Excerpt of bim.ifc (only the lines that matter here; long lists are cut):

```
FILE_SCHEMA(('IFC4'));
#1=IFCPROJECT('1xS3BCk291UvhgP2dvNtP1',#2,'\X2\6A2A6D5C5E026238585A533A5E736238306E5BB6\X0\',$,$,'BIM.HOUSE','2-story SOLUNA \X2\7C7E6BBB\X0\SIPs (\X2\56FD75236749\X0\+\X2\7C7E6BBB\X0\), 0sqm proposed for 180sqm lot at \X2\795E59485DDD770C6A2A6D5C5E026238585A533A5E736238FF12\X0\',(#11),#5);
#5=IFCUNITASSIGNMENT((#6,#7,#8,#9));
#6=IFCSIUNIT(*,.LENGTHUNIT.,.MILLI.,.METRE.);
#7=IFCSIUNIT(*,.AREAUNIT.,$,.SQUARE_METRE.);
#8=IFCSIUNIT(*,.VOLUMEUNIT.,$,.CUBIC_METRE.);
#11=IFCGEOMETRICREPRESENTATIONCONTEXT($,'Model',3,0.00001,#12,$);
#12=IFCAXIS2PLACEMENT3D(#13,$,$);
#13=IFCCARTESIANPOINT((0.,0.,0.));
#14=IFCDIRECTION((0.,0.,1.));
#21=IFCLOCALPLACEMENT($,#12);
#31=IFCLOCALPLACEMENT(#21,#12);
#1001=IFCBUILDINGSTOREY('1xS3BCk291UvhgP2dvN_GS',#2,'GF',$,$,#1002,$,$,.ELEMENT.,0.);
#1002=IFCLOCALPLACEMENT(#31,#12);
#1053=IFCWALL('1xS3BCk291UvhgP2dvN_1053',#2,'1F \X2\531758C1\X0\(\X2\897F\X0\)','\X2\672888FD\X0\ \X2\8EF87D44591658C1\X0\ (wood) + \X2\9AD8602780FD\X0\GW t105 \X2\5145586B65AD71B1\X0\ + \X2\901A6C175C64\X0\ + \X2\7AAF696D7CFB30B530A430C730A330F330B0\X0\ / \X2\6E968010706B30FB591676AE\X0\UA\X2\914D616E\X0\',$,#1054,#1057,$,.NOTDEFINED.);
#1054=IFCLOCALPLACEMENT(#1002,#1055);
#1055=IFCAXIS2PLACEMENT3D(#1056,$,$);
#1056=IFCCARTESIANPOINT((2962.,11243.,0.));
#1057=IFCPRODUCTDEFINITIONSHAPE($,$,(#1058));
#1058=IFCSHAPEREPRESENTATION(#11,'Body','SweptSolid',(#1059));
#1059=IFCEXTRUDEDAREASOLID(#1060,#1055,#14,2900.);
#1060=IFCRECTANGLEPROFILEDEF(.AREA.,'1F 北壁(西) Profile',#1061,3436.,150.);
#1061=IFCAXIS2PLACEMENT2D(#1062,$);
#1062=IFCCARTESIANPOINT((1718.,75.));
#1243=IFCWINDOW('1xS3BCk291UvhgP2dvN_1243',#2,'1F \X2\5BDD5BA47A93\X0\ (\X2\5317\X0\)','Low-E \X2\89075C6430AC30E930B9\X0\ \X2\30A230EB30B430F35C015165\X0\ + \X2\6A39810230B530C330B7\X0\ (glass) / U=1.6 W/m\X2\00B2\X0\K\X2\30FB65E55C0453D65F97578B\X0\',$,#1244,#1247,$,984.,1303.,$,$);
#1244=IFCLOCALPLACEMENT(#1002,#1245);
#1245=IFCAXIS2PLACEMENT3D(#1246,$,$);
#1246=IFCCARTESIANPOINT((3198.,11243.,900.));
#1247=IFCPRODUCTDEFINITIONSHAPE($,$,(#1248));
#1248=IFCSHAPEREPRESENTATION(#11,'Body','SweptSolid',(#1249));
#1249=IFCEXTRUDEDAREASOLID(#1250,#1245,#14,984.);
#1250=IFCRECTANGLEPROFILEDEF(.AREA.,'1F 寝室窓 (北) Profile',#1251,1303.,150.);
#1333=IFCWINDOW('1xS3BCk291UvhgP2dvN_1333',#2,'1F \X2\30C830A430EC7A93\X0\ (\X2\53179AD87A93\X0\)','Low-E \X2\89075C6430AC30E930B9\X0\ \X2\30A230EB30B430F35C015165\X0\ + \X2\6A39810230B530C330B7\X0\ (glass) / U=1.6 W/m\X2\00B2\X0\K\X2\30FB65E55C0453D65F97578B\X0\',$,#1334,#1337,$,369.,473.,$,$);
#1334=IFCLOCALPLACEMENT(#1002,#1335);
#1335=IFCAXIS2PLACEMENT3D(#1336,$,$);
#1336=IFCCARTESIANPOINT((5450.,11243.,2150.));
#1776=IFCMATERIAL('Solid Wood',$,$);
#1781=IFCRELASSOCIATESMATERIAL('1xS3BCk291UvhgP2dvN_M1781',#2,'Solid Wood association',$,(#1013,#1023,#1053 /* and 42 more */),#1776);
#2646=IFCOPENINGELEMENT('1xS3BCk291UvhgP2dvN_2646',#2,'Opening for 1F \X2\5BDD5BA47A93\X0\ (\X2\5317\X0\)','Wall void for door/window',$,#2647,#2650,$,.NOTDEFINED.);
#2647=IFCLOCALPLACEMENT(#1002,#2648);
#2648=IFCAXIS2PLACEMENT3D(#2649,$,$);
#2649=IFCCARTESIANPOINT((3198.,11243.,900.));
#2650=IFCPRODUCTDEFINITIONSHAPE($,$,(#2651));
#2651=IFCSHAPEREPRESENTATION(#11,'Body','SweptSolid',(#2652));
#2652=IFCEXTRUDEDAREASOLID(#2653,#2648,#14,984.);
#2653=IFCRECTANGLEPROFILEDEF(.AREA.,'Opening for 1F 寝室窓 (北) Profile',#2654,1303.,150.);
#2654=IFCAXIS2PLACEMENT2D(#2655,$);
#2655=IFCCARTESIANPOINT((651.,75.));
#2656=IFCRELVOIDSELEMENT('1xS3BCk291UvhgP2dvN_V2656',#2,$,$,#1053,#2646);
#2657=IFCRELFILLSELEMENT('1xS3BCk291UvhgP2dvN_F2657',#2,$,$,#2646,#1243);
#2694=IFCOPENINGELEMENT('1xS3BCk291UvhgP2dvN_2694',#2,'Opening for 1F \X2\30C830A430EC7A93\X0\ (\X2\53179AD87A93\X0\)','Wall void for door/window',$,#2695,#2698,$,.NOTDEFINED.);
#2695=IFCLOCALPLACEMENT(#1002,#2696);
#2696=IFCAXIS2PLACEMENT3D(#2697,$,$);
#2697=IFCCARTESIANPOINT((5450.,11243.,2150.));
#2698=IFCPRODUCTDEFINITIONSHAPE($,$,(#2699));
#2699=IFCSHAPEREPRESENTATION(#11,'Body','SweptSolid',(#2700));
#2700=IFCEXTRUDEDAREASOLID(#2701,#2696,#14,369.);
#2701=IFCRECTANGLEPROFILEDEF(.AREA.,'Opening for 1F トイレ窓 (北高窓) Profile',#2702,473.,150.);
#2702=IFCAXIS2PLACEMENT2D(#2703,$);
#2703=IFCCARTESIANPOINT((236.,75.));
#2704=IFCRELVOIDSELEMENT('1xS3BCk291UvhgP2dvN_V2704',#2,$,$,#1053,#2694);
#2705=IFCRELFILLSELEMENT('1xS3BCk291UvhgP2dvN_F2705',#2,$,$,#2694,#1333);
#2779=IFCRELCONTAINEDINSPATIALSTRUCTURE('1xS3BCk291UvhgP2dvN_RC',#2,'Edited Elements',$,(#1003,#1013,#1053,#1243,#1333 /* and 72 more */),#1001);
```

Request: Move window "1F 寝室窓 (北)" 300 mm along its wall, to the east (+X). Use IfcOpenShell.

```python
import ifcopenshell
import ifcopenshell.api.geometry
import ifcopenshell.util.placement

model = ifcopenshell.open("bim.ifc")

window = model.by_guid("1xS3BCk291UvhgP2dvN_1243")
opening = window.FillsVoids[0].RelatingOpeningElement
wall = opening.VoidsElements[0].RelatingBuildingElement

wall_matrix = ifcopenshell.util.placement.get_local_placement(wall.ObjectPlacement)
shift = wall_matrix[:3, 0] * 300.0
before = ifcopenshell.util.placement.get_local_placement(window.ObjectPlacement)[:3, 3].copy()

# The window is not placed relative to its opening, so move both.
for product in (opening, window):
    matrix = ifcopenshell.util.placement.get_local_placement(product.ObjectPlacement)
    matrix[:3, 3] += shift
    ifcopenshell.api.geometry.edit_object_placement(model, product=product, matrix=matrix, is_si=False)

after = ifcopenshell.util.placement.get_local_placement(window.ObjectPlacement)[:3, 3]
print("window moved by", (after - before).round(3) + 0.0)

model.write("bim_v2.ifc")
```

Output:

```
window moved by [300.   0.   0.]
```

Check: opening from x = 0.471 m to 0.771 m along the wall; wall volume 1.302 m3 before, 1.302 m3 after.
